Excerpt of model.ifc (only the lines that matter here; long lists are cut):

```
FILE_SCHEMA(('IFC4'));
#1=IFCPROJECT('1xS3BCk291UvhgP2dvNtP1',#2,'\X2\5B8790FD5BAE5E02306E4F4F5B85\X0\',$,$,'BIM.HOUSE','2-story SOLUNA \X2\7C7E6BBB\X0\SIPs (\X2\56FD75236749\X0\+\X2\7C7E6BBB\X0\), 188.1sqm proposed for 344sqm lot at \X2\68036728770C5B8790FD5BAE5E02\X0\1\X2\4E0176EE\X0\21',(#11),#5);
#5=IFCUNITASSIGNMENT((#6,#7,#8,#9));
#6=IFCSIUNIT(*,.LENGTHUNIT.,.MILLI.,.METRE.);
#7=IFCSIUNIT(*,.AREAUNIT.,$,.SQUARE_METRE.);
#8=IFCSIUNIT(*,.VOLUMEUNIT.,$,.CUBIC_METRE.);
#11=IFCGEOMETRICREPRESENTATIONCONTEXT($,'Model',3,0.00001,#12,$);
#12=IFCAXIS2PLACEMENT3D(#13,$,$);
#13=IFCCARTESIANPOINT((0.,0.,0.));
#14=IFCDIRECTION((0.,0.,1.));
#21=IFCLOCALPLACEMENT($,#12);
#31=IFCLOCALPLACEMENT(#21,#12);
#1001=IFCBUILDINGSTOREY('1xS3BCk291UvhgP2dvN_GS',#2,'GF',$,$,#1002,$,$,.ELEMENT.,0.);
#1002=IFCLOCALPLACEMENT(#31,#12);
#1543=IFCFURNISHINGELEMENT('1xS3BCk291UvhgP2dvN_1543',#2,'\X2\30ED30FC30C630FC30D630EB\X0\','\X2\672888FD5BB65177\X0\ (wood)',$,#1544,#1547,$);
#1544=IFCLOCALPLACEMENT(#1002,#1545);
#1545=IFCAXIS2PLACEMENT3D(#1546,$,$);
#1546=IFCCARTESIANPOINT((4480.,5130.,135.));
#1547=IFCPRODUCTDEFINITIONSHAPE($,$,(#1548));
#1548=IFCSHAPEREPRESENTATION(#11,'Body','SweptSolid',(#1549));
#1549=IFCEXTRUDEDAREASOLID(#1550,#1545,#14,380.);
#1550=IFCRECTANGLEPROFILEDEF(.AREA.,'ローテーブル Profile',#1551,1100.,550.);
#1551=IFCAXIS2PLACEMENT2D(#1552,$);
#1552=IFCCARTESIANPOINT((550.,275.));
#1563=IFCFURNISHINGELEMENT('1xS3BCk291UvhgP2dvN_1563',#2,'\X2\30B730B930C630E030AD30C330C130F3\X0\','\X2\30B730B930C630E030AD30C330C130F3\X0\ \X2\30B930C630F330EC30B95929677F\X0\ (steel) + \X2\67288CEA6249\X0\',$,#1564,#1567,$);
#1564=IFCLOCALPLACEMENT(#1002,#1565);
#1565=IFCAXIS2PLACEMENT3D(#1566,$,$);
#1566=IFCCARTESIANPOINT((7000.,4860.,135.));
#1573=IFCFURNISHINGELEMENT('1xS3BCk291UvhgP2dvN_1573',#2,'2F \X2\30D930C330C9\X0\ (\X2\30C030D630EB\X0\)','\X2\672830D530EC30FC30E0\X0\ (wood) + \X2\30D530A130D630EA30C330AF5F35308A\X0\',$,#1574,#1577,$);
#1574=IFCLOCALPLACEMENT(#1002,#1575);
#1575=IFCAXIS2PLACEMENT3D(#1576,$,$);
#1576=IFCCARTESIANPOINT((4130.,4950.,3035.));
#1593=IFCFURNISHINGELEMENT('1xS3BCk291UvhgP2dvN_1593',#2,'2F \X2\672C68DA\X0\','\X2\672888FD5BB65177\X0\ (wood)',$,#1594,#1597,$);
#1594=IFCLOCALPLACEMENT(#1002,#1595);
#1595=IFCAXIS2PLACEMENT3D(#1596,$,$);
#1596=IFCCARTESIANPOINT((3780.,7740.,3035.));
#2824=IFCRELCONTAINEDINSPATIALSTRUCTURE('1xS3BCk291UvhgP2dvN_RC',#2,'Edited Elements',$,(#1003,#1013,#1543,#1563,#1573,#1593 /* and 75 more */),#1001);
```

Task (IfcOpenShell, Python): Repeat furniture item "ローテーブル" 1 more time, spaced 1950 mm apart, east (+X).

```python
import numpy as np
import ifcopenshell
import ifcopenshell.api.geometry
import ifcopenshell.api.root
import ifcopenshell.util.element
import ifcopenshell.util.placement
import ifcopenshell.util.unit

model = ifcopenshell.open("model.ifc")
unit_scale = ifcopenshell.util.unit.calculate_unit_scale(model)


def reuse_history(source, copy):
    """copy_class also copies each property set's owner history, people and application; keep the originals."""
    for rel in copy.IsDefinedBy:
        if rel.is_a("IfcRelDefinesByProperties") and (history := rel.RelatingPropertyDefinition.OwnerHistory):
            rel.RelatingPropertyDefinition.OwnerHistory = source.OwnerHistory
            ifcopenshell.util.element.remove_deep2(model, history)


source = model.by_guid("1xS3BCk291UvhgP2dvN_1543")
base = ifcopenshell.util.placement.get_local_placement(source.ObjectPlacement)
step = np.array([1.0, 0.0, 0.0]) * 1.95 / unit_scale

for i in range(1, 2):
    copy = ifcopenshell.api.root.copy_class(model, product=source)
    copy.Representation = ifcopenshell.util.element.copy_deep(
        model, source.Representation, exclude=["IfcGeometricRepresentationContext", "IfcRepresentationMap"]
    )
    reuse_history(source, copy)
    matrix = base.copy()
    matrix[:3, 3] += i * step
    print("added at", matrix[:3, 3].round(3) + 0.0)
    ifcopenshell.api.geometry.edit_object_placement(model, product=copy, matrix=matrix, is_si=False)

model.write("model_rev.ifc")
```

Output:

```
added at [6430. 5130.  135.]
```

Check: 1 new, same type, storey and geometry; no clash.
